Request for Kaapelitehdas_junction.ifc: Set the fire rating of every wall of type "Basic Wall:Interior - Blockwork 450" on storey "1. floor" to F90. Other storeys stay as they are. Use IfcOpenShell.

First a look at what the model holds.

```python
import ifcopenshell
import ifcopenshell.util.element

model = ifcopenshell.open("Kaapelitehdas_junction.ifc")
print(model.schema)
storey = next(s for s in model.by_type("IfcBuildingStorey") if s.Name == "1. floor")
walls = [e for e in ifcopenshell.util.element.get_decomposition(storey) if e.is_a("IfcWall")]
seen = {}
for e in walls:
    element_type = ifcopenshell.util.element.get_type(e)
    key = (element_type.Name if element_type != e and element_type else None, ifcopenshell.util.element.get_pset(e, "Pset_WallCommon", "FireRating"))
    seen[key] = seen.get(key, 0) + 1
for (name, value), count in sorted(seen.items(), key=str):
    print(count, "x", name, "|", value)
```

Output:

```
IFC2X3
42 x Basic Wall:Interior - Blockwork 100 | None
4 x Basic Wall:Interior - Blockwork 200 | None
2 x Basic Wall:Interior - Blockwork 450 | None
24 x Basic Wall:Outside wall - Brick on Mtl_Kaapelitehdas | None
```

```python
import ifcopenshell
import ifcopenshell.api.pset
import ifcopenshell.util.element

model = ifcopenshell.open("Kaapelitehdas_junction.ifc")

storey = next(s for s in model.by_type("IfcBuildingStorey") if s.Name == "1. floor")
walls = [e for e in ifcopenshell.util.element.get_decomposition(storey) if e.is_a("IfcWall")]

count = 0
for e in walls:
    element_type = ifcopenshell.util.element.get_type(e)
    if element_type in (None, e) or element_type.Name != "Basic Wall:Interior - Blockwork 450":
        continue
    # add_pset returns the element's existing set when there is one.
    pset = ifcopenshell.api.pset.add_pset(model, product=e, name="Pset_WallCommon")
    ifcopenshell.api.pset.edit_pset(model, pset=pset, properties={"FireRating": "F90"})
    count += 1

print(count, "walls updated")

model.write("Kaapelitehdas_junction_v2.ifc")
```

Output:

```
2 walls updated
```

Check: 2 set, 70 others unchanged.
